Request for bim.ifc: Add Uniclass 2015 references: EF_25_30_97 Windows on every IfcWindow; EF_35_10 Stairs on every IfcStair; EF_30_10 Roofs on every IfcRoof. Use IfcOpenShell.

First a look at what the model holds.

```python
import ifcopenshell

model = ifcopenshell.open("bim.ifc")
print(model.schema)
print("classifications:", [c.Name for c in model.by_type("IfcClassification")])
for ifc_class in ("IfcDoor", "IfcRoof", "IfcStair", "IfcWall", "IfcWindow"):
    print(ifc_class, len(model.by_type(ifc_class)))
```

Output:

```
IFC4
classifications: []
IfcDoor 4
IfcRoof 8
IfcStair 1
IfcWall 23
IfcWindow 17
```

```python
import ifcopenshell
import ifcopenshell.api.classification

model = ifcopenshell.open("bim.ifc")

system = ifcopenshell.api.classification.add_classification(model, classification="Uniclass 2015")

codes = {
    "IfcWindow": ("EF_25_30_97", "Windows"),
    "IfcStair": ("EF_35_10", "Stairs"),
    "IfcRoof": ("EF_30_10", "Roofs"),
}
for ifc_class, (code, name) in codes.items():
    products = model.by_type(ifc_class)
    ifcopenshell.api.classification.add_reference(
        model, products=products, classification=system, identification=code, name=name
    )
    print(code, len(products))

model.write("bim_v2.ifc")
```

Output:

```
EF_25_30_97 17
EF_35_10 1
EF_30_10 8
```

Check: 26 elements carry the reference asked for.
